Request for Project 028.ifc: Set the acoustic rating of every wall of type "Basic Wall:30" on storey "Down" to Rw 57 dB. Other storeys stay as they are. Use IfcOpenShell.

First a look at what the model holds.

```python
import ifcopenshell
import ifcopenshell.util.element

model = ifcopenshell.open("Project 028.ifc")
print(model.schema)
storey = next(s for s in model.by_type("IfcBuildingStorey") if s.Name == "Down")
walls = [e for e in ifcopenshell.util.element.get_decomposition(storey) if e.is_a("IfcWall")]
seen = {}
for e in walls:
    element_type = ifcopenshell.util.element.get_type(e)
    key = (element_type.Name if element_type != e and element_type else None, ifcopenshell.util.element.get_pset(e, "Pset_WallCommon", "AcousticRating"))
    seen[key] = seen.get(key, 0) + 1
for (name, value), count in sorted(seen.items(), key=str):
    print(count, "x", name, "|", value)
```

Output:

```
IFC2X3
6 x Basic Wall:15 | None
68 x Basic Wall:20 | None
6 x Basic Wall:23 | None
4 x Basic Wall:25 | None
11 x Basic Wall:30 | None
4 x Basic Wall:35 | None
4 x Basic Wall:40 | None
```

```python
import ifcopenshell
import ifcopenshell.api.pset
import ifcopenshell.util.element

model = ifcopenshell.open("Project 028.ifc")

storey = next(s for s in model.by_type("IfcBuildingStorey") if s.Name == "Down")
walls = [e for e in ifcopenshell.util.element.get_decomposition(storey) if e.is_a("IfcWall")]

count = 0
for e in walls:
    element_type = ifcopenshell.util.element.get_type(e)
    if element_type in (None, e) or element_type.Name != "Basic Wall:30":
        continue
    # add_pset returns the element's existing set when there is one.
    pset = ifcopenshell.api.pset.add_pset(model, product=e, name="Pset_WallCommon")
    ifcopenshell.api.pset.edit_pset(model, pset=pset, properties={"AcousticRating": "Rw 57 dB"})
    count += 1

print(count, "walls updated")

model.write("Project 028_edited.ifc")
```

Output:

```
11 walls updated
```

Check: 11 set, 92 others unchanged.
